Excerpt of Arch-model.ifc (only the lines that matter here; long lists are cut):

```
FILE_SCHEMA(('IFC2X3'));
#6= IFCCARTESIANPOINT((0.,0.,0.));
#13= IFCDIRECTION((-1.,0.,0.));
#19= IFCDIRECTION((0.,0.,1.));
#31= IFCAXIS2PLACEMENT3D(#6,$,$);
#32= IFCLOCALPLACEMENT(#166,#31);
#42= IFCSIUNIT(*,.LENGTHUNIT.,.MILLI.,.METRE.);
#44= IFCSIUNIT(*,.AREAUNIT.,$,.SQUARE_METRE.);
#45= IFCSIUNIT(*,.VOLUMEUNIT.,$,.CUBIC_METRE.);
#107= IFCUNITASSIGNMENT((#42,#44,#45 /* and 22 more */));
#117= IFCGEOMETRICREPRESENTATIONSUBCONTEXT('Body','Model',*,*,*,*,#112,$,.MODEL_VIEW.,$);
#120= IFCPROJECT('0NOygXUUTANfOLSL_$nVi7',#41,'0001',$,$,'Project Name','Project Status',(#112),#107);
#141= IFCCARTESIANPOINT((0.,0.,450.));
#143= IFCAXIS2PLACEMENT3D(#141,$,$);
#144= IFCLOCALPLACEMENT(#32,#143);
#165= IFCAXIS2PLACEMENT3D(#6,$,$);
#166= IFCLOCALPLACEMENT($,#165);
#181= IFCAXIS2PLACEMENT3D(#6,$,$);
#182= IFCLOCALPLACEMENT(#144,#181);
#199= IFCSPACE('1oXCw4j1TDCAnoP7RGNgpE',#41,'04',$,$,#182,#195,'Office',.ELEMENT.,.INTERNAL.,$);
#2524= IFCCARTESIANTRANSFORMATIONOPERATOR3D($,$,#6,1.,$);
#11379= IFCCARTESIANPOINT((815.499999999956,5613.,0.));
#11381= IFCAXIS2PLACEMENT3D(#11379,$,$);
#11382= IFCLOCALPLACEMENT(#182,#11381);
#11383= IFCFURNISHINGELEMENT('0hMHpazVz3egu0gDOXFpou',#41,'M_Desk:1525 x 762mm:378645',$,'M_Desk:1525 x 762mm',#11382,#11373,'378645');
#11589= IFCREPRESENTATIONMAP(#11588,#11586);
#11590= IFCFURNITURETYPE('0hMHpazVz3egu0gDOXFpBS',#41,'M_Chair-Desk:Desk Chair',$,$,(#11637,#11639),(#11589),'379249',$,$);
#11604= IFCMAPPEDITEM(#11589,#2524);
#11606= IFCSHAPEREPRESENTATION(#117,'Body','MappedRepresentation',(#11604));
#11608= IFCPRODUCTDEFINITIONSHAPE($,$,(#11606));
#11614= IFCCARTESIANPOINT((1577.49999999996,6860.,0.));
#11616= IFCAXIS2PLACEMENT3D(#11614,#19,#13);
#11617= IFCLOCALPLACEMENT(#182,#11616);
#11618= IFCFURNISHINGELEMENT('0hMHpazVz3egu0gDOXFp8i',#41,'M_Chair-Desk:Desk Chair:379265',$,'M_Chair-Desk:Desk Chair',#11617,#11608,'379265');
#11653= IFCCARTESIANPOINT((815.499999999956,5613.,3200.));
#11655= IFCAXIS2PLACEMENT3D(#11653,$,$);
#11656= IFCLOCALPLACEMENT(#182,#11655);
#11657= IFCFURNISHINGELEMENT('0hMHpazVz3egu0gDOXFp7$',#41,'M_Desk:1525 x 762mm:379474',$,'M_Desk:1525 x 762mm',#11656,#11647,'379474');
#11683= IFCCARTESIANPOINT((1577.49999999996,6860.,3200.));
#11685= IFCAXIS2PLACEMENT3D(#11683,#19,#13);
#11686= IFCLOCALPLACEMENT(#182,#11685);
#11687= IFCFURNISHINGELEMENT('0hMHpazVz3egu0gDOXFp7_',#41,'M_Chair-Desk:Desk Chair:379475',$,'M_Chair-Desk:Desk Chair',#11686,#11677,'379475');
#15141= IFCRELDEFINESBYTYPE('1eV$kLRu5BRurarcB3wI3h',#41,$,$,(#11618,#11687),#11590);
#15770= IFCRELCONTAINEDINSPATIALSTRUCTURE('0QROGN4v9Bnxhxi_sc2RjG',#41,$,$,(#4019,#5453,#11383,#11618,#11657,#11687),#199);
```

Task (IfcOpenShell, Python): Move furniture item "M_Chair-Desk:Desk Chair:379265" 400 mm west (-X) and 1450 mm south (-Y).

```python
import ifcopenshell
import ifcopenshell.api.geometry
import ifcopenshell.util.placement

model = ifcopenshell.open("Arch-model.ifc")

item = model.by_id(11618)
matrix = ifcopenshell.util.placement.get_local_placement(item.ObjectPlacement)
matrix[0, 3] -= 400.0
matrix[1, 3] -= 1450.0
ifcopenshell.api.geometry.edit_object_placement(model, product=item, matrix=matrix, is_si=False)

print(ifcopenshell.util.placement.get_local_placement(item.ObjectPlacement).round(3) + 0.0)

model.write("Arch-model_rev.ifc")
```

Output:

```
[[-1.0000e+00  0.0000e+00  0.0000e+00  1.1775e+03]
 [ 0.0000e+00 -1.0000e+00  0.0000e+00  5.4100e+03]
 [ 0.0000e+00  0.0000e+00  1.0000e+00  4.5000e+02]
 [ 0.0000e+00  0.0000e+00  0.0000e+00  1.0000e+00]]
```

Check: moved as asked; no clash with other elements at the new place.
